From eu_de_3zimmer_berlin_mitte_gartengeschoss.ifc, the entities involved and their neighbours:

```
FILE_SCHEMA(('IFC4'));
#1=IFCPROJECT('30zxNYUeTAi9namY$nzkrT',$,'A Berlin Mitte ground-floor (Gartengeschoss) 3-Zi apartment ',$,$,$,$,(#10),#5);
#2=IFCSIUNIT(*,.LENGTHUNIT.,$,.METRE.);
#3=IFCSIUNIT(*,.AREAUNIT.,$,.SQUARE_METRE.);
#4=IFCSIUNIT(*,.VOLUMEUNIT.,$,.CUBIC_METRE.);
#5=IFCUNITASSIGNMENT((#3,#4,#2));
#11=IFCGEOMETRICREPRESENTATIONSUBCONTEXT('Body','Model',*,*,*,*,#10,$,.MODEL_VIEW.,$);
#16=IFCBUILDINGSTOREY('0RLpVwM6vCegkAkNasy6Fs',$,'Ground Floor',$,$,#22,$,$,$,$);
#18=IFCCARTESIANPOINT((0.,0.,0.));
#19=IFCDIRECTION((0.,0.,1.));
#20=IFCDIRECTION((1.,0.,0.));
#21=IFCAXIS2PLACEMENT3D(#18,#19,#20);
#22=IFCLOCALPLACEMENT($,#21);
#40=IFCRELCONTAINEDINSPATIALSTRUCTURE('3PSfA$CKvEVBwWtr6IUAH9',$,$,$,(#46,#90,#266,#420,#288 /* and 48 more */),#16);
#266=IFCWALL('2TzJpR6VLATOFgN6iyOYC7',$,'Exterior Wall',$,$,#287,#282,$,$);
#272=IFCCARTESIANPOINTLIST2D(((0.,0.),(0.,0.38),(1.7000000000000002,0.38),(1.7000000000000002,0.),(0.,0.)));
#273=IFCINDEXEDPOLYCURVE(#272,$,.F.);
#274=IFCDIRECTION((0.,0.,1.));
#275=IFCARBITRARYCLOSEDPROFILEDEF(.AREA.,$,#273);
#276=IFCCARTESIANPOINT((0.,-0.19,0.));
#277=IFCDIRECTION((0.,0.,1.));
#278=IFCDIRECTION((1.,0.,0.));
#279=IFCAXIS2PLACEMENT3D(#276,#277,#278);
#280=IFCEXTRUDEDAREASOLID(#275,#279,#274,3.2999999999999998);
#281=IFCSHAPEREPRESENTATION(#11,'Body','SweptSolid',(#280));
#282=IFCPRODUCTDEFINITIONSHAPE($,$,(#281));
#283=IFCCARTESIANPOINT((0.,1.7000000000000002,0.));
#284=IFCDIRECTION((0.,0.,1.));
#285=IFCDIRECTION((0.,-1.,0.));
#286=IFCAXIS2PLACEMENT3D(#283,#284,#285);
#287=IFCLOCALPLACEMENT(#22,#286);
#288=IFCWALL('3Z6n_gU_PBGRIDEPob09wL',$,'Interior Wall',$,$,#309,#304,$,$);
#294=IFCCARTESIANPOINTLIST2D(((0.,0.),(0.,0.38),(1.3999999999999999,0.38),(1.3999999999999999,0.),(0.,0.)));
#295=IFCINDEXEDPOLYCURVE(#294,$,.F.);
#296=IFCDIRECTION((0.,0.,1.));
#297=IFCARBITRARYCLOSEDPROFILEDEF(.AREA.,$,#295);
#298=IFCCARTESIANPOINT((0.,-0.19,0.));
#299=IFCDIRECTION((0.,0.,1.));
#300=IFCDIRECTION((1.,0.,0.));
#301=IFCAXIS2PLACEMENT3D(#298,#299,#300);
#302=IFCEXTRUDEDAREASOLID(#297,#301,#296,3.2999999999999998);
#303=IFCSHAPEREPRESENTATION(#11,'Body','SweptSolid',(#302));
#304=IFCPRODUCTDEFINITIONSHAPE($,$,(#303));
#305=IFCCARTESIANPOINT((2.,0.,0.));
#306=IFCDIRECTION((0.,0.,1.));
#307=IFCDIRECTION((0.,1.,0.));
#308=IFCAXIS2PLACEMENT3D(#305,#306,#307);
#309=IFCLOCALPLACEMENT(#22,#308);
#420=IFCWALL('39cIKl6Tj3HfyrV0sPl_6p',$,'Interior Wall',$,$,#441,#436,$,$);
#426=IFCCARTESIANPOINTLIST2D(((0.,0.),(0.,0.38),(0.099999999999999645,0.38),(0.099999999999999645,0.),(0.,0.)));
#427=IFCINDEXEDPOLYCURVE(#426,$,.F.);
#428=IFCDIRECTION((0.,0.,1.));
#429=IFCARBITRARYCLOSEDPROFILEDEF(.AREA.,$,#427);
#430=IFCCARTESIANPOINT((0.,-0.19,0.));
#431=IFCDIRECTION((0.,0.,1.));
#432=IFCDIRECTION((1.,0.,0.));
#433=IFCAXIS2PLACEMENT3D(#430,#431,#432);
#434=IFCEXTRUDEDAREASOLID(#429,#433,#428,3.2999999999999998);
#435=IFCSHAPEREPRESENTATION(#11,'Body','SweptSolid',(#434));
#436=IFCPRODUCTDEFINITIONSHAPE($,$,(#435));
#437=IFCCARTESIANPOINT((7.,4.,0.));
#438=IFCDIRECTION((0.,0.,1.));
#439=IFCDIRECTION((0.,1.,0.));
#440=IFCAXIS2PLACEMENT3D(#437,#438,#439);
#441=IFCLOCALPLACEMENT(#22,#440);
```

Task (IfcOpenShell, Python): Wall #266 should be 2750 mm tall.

```python
import ifcopenshell
import ifcopenshell.geom
import ifcopenshell.util.representation
import ifcopenshell.util.shape

model = ifcopenshell.open("eu_de_3zimmer_berlin_mitte_gartengeschoss.ifc")
settings = ifcopenshell.geom.settings()


def volume(element):
    """Net volume in cubic metres, openings subtracted."""
    shape = ifcopenshell.geom.create_shape(settings, element)
    return ifcopenshell.util.shape.get_volume(shape.geometry)


wall = model.by_guid("2TzJpR6VLATOFgN6iyOYC7")
before = volume(wall)

body = ifcopenshell.util.representation.get_representation(wall, "Model", "Body")
solid = body.Items[0]
old_height = solid.Depth
solid.Depth = 2.75
after = volume(wall)

print(f"height {old_height:g} -> {solid.Depth:g}, volume {before:.3f} -> {after:.3f} m3")

model.write("eu_de_3zimmer_berlin_mitte_gartengeschoss_edited.ifc")
```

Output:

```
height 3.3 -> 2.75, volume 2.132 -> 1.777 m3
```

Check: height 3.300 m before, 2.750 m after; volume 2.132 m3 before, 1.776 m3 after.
